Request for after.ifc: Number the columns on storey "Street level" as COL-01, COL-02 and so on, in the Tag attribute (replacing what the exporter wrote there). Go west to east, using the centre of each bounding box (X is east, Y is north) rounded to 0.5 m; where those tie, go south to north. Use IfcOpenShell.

First a look at what the model holds.

```python
import ifcopenshell
import ifcopenshell.util.element
import ifcopenshell.util.placement

model = ifcopenshell.open("after.ifc")
print(model.schema)
storey = next(s for s in model.by_type("IfcBuildingStorey") if s.Name == "Street level")
columns = [e for e in ifcopenshell.util.element.get_decomposition(storey) if e.is_a("IfcColumn")]
for e in sorted(columns, key=lambda e: e.id()):
    origin = ifcopenshell.util.placement.get_local_placement(e.ObjectPlacement)[:3, 3]
    print(e.id(), e.Tag, e.Name, origin.round(2) + 0.0, sep=" | ")
```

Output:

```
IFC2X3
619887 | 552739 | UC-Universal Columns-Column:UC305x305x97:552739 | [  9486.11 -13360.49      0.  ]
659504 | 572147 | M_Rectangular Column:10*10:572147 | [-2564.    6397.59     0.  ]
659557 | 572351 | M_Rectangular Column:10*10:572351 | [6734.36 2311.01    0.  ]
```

```python
import ifcopenshell
import ifcopenshell.geom
import ifcopenshell.util.element
import ifcopenshell.util.shape

model = ifcopenshell.open("after.ifc")
settings = ifcopenshell.geom.settings()
settings.set("use-world-coords", True)


def centre(element):
    shape = ifcopenshell.geom.create_shape(settings, element)
    return ifcopenshell.util.shape.get_bbox_centroid(shape.geometry)


storey = next(s for s in model.by_type("IfcBuildingStorey") if s.Name == "Street level")
columns = [e for e in ifcopenshell.util.element.get_decomposition(storey) if e.is_a("IfcColumn")]

# Insertion points can sit at a corner or the storey origin, so sort by the geometry (in metres).
centres = {e: centre(e) for e in columns}
columns.sort(key=lambda e: (round(centres[e][0] / 0.5), centres[e][1]))

for i, e in enumerate(columns, start=1):
    number = f"COL-{i:02d}"
    e.Tag = number
    print(e.id(), number)

model.write("after_updated.ifc")
```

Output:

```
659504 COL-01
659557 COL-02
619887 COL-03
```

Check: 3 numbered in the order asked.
